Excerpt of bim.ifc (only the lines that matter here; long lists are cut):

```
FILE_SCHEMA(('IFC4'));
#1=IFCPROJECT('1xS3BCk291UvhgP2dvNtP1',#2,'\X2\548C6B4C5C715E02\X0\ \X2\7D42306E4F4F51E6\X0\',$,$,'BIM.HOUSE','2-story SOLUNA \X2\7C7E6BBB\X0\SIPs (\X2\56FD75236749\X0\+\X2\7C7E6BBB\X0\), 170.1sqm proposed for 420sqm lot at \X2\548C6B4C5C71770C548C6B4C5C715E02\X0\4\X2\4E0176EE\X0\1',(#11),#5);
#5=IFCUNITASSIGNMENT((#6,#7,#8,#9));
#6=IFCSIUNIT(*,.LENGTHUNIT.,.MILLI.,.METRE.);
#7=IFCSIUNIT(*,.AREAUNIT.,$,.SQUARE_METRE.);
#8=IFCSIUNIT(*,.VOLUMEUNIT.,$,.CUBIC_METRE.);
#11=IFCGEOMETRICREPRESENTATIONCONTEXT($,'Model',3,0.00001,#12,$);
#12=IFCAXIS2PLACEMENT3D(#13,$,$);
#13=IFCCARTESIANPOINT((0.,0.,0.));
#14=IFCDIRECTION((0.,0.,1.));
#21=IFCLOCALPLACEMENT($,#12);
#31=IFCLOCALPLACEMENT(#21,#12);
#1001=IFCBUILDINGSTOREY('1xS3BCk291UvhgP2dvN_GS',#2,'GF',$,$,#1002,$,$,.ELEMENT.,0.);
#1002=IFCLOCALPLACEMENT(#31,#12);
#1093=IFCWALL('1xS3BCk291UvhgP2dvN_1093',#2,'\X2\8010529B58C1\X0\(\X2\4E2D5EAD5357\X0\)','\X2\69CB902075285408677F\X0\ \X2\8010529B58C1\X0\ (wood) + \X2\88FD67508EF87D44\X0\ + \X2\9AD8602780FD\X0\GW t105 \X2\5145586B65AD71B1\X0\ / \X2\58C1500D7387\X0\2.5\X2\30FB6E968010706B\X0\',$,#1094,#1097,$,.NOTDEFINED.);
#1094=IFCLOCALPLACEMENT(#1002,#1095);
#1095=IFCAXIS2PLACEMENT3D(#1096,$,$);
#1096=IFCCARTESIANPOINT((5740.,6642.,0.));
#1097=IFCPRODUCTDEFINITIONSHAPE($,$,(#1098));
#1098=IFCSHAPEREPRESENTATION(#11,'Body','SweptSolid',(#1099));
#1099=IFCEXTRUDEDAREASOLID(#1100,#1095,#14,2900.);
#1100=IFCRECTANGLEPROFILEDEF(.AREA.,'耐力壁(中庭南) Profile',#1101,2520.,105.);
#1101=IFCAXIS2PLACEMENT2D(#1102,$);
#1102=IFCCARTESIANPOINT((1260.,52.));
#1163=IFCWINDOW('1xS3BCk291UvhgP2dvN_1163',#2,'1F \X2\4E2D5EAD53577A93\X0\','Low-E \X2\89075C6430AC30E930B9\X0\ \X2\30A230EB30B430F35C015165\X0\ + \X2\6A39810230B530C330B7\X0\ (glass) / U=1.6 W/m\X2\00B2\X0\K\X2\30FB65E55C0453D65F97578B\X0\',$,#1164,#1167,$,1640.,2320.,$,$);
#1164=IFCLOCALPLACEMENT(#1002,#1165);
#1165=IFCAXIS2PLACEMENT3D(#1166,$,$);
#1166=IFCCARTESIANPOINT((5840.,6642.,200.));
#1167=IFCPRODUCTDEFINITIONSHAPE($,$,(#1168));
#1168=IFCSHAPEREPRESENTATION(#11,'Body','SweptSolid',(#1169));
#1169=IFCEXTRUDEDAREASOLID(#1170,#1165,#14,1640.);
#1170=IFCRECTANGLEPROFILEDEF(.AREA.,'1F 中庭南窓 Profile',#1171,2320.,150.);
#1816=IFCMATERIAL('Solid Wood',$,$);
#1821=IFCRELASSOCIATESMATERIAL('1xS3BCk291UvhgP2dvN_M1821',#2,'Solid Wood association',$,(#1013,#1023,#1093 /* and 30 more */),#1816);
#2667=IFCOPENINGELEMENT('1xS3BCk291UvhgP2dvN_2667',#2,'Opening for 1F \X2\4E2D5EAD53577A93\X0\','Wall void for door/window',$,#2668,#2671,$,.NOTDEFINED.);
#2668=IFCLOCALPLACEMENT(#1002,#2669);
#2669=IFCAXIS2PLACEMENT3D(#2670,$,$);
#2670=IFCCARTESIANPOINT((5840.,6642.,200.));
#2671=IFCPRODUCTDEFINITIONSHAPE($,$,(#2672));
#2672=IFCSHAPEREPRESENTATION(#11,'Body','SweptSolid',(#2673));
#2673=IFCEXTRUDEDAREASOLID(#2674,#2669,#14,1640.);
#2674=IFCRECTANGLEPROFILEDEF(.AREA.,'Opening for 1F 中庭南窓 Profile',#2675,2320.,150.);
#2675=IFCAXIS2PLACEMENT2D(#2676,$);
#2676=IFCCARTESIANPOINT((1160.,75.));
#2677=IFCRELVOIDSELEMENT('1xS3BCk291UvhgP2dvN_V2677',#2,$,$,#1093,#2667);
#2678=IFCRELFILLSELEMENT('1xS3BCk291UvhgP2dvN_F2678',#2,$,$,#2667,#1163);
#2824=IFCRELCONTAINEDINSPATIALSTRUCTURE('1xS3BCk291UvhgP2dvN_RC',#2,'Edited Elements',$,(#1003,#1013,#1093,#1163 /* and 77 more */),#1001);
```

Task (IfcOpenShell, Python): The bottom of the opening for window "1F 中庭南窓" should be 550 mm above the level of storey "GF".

```python
import numpy as np
import ifcopenshell
import ifcopenshell.api.geometry
import ifcopenshell.geom
import ifcopenshell.util.element
import ifcopenshell.util.placement
import ifcopenshell.util.shape
import ifcopenshell.util.unit

model = ifcopenshell.open("bim.ifc")
unit_scale = ifcopenshell.util.unit.calculate_unit_scale(model)

window = model.by_guid("1xS3BCk291UvhgP2dvN_1163")
opening = window.FillsVoids[0].RelatingOpeningElement
storey = ifcopenshell.util.element.get_container(window, ifc_class="IfcBuildingStorey")
level = ifcopenshell.util.placement.get_local_placement(storey.ObjectPlacement)[2, 3]

# The opening's origin need not be at the sill, so measure its lowest point.
shape = ifcopenshell.geom.create_shape(ifcopenshell.geom.settings(), opening)
bottom = ifcopenshell.util.shape.get_shape_bottom_elevation(shape, shape.geometry) / unit_scale
dz = level + 0.55 / unit_scale - bottom

shift = np.array([0.0, 0.0, dz])
# The window is not placed relative to its opening, so move both.
for product in (opening, window):
    matrix = ifcopenshell.util.placement.get_local_placement(product.ObjectPlacement)
    matrix[:3, 3] += shift
    ifcopenshell.api.geometry.edit_object_placement(model, product=product, matrix=matrix, is_si=False)

print(f"moved by {dz * unit_scale:+.3f} m")

model.write("bim_rev.ifc")
```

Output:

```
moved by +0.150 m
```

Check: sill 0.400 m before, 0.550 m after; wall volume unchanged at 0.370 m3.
